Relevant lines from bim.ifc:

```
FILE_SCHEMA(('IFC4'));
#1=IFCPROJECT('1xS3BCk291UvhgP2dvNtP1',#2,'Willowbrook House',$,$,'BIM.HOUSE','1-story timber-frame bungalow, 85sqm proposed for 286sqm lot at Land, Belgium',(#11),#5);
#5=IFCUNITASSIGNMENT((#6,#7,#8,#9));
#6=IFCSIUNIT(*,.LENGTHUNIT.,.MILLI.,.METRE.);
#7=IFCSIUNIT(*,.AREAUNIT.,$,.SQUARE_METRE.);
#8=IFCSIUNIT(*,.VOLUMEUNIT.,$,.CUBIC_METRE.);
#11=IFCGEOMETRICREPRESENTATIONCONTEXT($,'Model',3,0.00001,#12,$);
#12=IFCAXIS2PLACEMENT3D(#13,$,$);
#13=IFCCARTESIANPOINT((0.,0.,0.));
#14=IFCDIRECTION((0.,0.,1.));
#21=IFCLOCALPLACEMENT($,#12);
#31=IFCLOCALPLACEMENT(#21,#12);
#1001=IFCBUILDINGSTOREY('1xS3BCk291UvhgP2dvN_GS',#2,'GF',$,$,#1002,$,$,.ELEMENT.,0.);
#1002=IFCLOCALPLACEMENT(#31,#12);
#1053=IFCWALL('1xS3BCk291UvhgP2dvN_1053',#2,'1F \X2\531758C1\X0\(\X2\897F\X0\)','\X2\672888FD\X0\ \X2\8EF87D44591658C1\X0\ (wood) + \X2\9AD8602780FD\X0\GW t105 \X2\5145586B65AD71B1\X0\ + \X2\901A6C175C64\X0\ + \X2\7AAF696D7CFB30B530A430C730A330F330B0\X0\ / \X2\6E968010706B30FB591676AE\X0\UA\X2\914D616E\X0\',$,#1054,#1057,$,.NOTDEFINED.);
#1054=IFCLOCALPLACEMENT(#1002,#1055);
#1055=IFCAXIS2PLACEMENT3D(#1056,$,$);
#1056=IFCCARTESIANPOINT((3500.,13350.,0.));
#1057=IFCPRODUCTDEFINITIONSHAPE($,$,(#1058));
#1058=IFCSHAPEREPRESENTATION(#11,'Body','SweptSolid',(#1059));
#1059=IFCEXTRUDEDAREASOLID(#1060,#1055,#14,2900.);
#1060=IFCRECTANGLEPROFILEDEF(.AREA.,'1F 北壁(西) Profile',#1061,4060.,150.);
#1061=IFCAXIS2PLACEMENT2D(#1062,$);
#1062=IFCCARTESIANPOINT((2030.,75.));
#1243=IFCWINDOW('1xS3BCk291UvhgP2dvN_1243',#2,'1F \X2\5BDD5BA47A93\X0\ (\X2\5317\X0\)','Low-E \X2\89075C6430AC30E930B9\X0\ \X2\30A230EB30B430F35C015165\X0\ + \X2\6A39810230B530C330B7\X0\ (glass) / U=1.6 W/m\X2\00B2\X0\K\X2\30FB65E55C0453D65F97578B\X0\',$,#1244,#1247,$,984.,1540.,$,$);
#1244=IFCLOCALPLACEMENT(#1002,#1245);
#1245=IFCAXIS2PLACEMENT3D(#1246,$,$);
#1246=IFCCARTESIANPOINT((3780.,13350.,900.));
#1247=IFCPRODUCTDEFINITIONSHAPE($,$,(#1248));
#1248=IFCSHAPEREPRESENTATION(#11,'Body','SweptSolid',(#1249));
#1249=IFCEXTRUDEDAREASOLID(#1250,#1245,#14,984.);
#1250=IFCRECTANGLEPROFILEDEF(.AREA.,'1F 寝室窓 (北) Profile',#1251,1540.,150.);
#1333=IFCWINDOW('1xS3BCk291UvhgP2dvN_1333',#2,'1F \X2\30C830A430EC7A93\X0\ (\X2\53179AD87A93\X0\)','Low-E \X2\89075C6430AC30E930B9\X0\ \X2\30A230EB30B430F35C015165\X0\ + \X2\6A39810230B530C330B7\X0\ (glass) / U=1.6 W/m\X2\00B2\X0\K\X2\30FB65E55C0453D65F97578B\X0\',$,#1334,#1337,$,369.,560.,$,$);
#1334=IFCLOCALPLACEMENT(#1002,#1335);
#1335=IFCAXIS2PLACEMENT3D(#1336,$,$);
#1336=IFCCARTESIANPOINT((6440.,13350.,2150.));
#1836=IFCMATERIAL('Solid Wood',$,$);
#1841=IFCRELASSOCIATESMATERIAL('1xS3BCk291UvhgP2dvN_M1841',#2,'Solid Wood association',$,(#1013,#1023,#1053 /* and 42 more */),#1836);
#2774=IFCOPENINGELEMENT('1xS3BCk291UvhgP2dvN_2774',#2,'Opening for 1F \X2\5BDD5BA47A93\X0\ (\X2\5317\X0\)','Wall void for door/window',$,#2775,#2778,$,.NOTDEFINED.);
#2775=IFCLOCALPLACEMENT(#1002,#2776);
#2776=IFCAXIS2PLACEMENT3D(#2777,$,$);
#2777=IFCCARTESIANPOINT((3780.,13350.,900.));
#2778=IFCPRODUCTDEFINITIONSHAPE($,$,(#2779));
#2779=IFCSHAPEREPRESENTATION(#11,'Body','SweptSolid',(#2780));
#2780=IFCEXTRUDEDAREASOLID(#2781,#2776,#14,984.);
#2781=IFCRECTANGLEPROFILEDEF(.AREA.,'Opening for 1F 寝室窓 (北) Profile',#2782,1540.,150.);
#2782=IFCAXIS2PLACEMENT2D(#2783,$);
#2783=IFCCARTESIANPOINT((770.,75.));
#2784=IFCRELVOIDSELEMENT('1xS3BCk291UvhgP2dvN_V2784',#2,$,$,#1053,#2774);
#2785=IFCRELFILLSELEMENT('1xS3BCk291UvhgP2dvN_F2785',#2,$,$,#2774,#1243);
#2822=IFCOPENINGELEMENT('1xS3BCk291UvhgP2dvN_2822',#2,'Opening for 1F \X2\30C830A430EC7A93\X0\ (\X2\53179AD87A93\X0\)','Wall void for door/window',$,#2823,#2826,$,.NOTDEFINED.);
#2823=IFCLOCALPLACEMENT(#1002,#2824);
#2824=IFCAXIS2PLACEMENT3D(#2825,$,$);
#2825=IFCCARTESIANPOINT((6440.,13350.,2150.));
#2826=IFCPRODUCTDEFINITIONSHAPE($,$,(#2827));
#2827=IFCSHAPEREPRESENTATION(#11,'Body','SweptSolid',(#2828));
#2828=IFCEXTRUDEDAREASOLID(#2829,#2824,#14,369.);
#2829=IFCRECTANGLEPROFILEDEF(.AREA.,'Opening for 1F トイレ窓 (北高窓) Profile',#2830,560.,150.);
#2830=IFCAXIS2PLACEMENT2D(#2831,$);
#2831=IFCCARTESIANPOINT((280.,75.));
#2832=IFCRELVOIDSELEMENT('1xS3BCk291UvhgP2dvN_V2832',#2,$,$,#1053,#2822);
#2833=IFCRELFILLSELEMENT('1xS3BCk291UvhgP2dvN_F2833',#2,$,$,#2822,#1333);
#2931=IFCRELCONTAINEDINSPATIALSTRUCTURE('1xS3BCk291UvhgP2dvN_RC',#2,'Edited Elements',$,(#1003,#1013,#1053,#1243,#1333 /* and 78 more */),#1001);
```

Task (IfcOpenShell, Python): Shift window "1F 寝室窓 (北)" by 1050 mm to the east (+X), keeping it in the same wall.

```python
import ifcopenshell
import ifcopenshell.api.geometry
import ifcopenshell.util.placement

model = ifcopenshell.open("bim.ifc")

window = model.by_guid("1xS3BCk291UvhgP2dvN_1243")
opening = window.FillsVoids[0].RelatingOpeningElement
wall = opening.VoidsElements[0].RelatingBuildingElement

wall_matrix = ifcopenshell.util.placement.get_local_placement(wall.ObjectPlacement)
shift = wall_matrix[:3, 0] * 1050.0
before = ifcopenshell.util.placement.get_local_placement(window.ObjectPlacement)[:3, 3].copy()

# The window is not placed relative to its opening, so move both.
for product in (opening, window):
    matrix = ifcopenshell.util.placement.get_local_placement(product.ObjectPlacement)
    matrix[:3, 3] += shift
    ifcopenshell.api.geometry.edit_object_placement(model, product=product, matrix=matrix, is_si=False)

after = ifcopenshell.util.placement.get_local_placement(window.ObjectPlacement)[:3, 3]
print("window moved by", (after - before).round(3) + 0.0)

model.write("bim_edited.ifc")
```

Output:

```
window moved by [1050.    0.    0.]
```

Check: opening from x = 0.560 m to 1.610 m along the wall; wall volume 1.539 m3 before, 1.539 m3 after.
